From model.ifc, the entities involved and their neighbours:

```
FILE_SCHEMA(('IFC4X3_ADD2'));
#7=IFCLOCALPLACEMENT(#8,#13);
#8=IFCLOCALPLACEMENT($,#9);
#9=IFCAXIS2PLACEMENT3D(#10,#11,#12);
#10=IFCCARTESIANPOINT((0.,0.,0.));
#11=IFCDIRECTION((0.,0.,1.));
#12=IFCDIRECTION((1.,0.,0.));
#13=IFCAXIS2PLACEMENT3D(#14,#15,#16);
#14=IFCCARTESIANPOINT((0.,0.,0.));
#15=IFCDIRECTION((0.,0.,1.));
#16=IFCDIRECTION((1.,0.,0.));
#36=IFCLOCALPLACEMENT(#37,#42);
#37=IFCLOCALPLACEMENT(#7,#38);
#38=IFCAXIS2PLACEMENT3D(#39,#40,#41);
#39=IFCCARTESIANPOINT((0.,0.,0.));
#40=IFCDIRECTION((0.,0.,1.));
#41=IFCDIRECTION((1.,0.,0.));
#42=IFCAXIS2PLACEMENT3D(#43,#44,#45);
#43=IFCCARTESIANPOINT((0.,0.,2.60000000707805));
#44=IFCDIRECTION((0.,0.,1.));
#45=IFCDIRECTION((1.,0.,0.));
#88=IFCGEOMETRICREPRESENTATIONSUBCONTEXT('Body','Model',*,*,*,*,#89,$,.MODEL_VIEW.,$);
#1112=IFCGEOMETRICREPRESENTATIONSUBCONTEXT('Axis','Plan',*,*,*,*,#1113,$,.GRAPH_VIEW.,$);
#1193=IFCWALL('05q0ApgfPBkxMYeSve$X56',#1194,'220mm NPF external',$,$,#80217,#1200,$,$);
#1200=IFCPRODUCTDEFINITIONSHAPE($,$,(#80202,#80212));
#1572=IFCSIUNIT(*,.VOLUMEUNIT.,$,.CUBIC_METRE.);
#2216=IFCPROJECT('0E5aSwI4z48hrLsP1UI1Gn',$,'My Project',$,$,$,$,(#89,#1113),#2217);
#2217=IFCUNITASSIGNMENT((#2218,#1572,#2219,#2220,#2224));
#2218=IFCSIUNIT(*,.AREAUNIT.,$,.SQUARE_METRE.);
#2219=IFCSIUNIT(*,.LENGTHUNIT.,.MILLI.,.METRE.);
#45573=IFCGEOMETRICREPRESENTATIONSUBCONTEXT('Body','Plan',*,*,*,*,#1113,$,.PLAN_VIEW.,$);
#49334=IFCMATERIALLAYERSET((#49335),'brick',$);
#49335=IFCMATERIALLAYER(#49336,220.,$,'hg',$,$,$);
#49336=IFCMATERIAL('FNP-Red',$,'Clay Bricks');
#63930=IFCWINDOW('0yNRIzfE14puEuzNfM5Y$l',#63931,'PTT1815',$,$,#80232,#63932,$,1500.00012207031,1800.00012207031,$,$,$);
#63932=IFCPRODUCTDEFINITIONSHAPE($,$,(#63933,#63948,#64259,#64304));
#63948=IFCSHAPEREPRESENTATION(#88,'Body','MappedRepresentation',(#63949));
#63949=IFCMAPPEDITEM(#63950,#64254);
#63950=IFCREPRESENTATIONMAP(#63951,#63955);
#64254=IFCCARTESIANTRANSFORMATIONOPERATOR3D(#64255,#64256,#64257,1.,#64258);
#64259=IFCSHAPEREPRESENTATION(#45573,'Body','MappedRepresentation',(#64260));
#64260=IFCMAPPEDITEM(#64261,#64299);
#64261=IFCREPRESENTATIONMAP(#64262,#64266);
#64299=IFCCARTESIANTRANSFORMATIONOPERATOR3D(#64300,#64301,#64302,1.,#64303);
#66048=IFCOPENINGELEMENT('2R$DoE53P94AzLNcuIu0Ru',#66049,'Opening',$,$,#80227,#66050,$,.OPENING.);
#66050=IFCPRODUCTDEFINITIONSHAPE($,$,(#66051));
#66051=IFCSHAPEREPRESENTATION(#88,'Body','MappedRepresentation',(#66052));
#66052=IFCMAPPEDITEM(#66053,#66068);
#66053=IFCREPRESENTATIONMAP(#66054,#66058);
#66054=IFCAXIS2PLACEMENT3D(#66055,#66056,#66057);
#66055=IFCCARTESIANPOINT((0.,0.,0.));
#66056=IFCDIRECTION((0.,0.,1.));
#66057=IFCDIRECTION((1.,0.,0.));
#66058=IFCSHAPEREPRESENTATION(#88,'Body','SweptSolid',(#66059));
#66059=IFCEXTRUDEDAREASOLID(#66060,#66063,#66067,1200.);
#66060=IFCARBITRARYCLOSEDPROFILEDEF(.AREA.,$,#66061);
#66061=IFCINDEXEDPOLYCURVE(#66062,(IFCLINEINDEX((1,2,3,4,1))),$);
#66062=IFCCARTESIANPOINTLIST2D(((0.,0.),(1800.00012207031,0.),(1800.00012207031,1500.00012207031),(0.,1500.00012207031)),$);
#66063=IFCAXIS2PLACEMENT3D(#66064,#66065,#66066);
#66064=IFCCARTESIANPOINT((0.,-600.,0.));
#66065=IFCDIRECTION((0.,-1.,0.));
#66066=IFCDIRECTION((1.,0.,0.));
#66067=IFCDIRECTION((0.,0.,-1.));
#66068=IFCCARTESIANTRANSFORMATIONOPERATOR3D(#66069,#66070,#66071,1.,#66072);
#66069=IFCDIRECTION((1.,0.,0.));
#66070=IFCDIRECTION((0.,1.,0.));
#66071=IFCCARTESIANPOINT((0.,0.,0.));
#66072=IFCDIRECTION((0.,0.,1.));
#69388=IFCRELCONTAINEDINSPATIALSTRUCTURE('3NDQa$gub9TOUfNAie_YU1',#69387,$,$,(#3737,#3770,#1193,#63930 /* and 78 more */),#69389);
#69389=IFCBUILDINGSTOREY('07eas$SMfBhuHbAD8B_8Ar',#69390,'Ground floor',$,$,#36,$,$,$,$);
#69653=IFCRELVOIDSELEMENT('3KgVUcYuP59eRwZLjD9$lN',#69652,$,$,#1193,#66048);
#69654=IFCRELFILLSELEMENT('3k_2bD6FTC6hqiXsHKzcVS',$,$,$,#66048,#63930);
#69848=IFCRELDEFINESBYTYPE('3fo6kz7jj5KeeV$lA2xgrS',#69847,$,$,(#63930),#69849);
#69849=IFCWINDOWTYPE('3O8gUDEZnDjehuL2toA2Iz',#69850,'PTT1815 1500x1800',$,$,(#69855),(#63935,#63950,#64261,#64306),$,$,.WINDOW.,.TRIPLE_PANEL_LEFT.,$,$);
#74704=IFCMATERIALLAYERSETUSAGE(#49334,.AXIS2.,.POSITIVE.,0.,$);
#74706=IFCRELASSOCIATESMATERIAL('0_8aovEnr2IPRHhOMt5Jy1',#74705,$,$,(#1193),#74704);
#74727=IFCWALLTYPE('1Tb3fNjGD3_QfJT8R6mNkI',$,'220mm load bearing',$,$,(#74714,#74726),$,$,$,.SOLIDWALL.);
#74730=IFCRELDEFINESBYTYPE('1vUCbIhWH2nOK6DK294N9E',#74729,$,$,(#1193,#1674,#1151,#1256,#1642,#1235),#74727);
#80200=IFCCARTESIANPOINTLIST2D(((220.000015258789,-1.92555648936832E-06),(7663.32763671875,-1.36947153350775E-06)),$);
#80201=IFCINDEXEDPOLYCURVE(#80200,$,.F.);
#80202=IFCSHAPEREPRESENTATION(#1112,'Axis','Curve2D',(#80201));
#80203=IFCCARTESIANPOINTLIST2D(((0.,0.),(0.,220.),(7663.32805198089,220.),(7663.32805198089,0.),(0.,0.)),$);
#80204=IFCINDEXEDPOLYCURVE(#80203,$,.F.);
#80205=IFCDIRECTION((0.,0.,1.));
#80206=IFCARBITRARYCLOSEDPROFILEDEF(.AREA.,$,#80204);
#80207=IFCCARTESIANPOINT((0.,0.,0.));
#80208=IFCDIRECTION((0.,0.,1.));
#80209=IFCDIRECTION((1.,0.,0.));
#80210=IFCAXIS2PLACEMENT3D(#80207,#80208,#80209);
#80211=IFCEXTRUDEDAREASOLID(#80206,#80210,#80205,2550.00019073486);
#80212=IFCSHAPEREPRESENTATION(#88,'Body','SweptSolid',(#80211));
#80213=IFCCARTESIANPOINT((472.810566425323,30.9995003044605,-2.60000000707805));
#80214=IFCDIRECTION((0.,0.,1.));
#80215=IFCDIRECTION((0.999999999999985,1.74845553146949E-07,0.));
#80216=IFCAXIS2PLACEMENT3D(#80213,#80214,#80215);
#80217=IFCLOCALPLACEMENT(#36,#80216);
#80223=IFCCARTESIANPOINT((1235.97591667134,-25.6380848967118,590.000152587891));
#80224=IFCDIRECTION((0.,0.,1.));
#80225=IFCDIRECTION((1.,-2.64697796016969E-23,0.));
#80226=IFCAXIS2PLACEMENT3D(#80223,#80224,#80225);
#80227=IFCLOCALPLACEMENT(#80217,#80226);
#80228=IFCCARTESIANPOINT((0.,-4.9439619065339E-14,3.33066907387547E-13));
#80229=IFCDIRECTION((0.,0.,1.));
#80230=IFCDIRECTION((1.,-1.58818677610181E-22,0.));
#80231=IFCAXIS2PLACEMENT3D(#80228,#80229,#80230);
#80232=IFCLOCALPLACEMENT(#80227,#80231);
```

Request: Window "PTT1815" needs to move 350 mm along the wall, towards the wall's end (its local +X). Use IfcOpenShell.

```python
import ifcopenshell
import ifcopenshell.api.geometry
import ifcopenshell.util.placement
import ifcopenshell.util.unit

model = ifcopenshell.open("model.ifc")
unit_scale = ifcopenshell.util.unit.calculate_unit_scale(model)

window = model.by_guid("0yNRIzfE14puEuzNfM5Y$l")
opening = window.FillsVoids[0].RelatingOpeningElement
wall = opening.VoidsElements[0].RelatingBuildingElement

wall_matrix = ifcopenshell.util.placement.get_local_placement(wall.ObjectPlacement)
shift = wall_matrix[:3, 0] * 0.35 / unit_scale
before = ifcopenshell.util.placement.get_local_placement(window.ObjectPlacement)[:3, 3].copy()

# The window is placed relative to its opening, so it follows when the opening moves.
matrix = ifcopenshell.util.placement.get_local_placement(opening.ObjectPlacement)
matrix[:3, 3] += shift
ifcopenshell.api.geometry.edit_object_placement(
    model, product=opening, matrix=matrix, is_si=False, should_transform_children=True
)

after = ifcopenshell.util.placement.get_local_placement(window.ObjectPlacement)[:3, 3]
print("window moved by", (after - before).round(3) + 0.0)

model.write("model_v2.ifc")
```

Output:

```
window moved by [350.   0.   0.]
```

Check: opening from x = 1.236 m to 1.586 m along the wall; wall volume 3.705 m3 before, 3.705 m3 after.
